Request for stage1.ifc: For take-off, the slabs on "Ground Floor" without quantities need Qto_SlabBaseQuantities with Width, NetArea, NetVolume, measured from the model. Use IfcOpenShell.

First a look at what the model holds.

```python
import ifcopenshell
import ifcopenshell.util.element
import ifcopenshell.util.unit

model = ifcopenshell.open("stage1.ifc")
print(model.schema)
for unit_type in ("LENGTHUNIT", "AREAUNIT", "VOLUMEUNIT"):
    print(unit_type, ifcopenshell.util.unit.calculate_unit_scale(model, unit_type))
storey = next(s for s in model.by_type("IfcBuildingStorey") if s.Name == "Ground Floor")
slabs = [e for e in ifcopenshell.util.element.get_decomposition(storey) if e.is_a("IfcSlab")]
for e in sorted(slabs, key=lambda e: e.id()):
    print(e.id(), e.is_a(), e.Name, list(ifcopenshell.util.element.get_psets(e, qtos_only=True)), sep=" | ")
```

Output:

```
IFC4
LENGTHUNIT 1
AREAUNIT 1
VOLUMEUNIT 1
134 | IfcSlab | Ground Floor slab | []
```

```python
import ifcopenshell
import ifcopenshell.api.pset
import ifcopenshell.geom
import ifcopenshell.util.element
import ifcopenshell.util.shape
import ifcopenshell.util.unit

model = ifcopenshell.open("stage1.ifc")
unit_scale = ifcopenshell.util.unit.calculate_unit_scale(model)
area_scale = ifcopenshell.util.unit.calculate_unit_scale(model, "AREAUNIT")
volume_scale = ifcopenshell.util.unit.calculate_unit_scale(model, "VOLUMEUNIT")
settings = ifcopenshell.geom.settings()

storey = next(s for s in model.by_type("IfcBuildingStorey") if s.Name == "Ground Floor")
slabs = [e for e in ifcopenshell.util.element.get_decomposition(storey) if e.is_a("IfcSlab")]

for e in sorted(slabs, key=lambda e: e.id()):
    if ifcopenshell.util.element.get_psets(e, qtos_only=True, should_inherit=False):
        continue
    # Geometry comes back in metres, in the element's own axes.
    shape = ifcopenshell.geom.create_shape(settings, e)
    values = {
        "Width": ifcopenshell.util.shape.get_z(shape.geometry) / unit_scale,
        "NetArea": ifcopenshell.util.shape.get_footprint_area(shape.geometry) / area_scale,
        "NetVolume": ifcopenshell.util.shape.get_volume(shape.geometry) / volume_scale,
    }
    qto = ifcopenshell.api.pset.add_qto(model, product=e, name="Qto_SlabBaseQuantities")
    ifcopenshell.api.pset.edit_qto(model, qto=qto, properties=values)
    print(e.id(), {k: round(v, 3) for k, v in values.items()})

model.write("stage1_updated.ifc")
```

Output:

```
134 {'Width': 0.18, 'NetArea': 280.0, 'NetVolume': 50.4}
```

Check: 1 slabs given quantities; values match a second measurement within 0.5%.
